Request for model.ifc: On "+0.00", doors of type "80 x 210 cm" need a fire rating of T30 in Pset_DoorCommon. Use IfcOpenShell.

First a look at what the model holds.

```python
import ifcopenshell
import ifcopenshell.util.element

model = ifcopenshell.open("model.ifc")
print(model.schema)
storey = next(s for s in model.by_type("IfcBuildingStorey") if s.Name == "+0.00")
doors = [e for e in ifcopenshell.util.element.get_decomposition(storey) if e.is_a("IfcDoor")]
seen = {}
for e in doors:
    element_type = ifcopenshell.util.element.get_type(e)
    key = (element_type.Name if element_type != e and element_type else None, ifcopenshell.util.element.get_pset(e, "Pset_DoorCommon", "FireRating"))
    seen[key] = seen.get(key, 0) + 1
for (name, value), count in sorted(seen.items(), key=str):
    print(count, "x", name, "|", value)
```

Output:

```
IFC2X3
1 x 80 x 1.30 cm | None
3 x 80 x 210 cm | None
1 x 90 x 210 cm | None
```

```python
import ifcopenshell
import ifcopenshell.api.pset
import ifcopenshell.util.element

model = ifcopenshell.open("model.ifc")

storey = next(s for s in model.by_type("IfcBuildingStorey") if s.Name == "+0.00")
doors = [e for e in ifcopenshell.util.element.get_decomposition(storey) if e.is_a("IfcDoor")]

count = 0
for e in doors:
    element_type = ifcopenshell.util.element.get_type(e)
    if element_type in (None, e) or element_type.Name != "80 x 210 cm":
        continue
    # add_pset returns the element's existing set when there is one.
    pset = ifcopenshell.api.pset.add_pset(model, product=e, name="Pset_DoorCommon")
    ifcopenshell.api.pset.edit_pset(model, pset=pset, properties={"FireRating": "T30"})
    count += 1

print(count, "doors updated")

model.write("model_updated.ifc")
```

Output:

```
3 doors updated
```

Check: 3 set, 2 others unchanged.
